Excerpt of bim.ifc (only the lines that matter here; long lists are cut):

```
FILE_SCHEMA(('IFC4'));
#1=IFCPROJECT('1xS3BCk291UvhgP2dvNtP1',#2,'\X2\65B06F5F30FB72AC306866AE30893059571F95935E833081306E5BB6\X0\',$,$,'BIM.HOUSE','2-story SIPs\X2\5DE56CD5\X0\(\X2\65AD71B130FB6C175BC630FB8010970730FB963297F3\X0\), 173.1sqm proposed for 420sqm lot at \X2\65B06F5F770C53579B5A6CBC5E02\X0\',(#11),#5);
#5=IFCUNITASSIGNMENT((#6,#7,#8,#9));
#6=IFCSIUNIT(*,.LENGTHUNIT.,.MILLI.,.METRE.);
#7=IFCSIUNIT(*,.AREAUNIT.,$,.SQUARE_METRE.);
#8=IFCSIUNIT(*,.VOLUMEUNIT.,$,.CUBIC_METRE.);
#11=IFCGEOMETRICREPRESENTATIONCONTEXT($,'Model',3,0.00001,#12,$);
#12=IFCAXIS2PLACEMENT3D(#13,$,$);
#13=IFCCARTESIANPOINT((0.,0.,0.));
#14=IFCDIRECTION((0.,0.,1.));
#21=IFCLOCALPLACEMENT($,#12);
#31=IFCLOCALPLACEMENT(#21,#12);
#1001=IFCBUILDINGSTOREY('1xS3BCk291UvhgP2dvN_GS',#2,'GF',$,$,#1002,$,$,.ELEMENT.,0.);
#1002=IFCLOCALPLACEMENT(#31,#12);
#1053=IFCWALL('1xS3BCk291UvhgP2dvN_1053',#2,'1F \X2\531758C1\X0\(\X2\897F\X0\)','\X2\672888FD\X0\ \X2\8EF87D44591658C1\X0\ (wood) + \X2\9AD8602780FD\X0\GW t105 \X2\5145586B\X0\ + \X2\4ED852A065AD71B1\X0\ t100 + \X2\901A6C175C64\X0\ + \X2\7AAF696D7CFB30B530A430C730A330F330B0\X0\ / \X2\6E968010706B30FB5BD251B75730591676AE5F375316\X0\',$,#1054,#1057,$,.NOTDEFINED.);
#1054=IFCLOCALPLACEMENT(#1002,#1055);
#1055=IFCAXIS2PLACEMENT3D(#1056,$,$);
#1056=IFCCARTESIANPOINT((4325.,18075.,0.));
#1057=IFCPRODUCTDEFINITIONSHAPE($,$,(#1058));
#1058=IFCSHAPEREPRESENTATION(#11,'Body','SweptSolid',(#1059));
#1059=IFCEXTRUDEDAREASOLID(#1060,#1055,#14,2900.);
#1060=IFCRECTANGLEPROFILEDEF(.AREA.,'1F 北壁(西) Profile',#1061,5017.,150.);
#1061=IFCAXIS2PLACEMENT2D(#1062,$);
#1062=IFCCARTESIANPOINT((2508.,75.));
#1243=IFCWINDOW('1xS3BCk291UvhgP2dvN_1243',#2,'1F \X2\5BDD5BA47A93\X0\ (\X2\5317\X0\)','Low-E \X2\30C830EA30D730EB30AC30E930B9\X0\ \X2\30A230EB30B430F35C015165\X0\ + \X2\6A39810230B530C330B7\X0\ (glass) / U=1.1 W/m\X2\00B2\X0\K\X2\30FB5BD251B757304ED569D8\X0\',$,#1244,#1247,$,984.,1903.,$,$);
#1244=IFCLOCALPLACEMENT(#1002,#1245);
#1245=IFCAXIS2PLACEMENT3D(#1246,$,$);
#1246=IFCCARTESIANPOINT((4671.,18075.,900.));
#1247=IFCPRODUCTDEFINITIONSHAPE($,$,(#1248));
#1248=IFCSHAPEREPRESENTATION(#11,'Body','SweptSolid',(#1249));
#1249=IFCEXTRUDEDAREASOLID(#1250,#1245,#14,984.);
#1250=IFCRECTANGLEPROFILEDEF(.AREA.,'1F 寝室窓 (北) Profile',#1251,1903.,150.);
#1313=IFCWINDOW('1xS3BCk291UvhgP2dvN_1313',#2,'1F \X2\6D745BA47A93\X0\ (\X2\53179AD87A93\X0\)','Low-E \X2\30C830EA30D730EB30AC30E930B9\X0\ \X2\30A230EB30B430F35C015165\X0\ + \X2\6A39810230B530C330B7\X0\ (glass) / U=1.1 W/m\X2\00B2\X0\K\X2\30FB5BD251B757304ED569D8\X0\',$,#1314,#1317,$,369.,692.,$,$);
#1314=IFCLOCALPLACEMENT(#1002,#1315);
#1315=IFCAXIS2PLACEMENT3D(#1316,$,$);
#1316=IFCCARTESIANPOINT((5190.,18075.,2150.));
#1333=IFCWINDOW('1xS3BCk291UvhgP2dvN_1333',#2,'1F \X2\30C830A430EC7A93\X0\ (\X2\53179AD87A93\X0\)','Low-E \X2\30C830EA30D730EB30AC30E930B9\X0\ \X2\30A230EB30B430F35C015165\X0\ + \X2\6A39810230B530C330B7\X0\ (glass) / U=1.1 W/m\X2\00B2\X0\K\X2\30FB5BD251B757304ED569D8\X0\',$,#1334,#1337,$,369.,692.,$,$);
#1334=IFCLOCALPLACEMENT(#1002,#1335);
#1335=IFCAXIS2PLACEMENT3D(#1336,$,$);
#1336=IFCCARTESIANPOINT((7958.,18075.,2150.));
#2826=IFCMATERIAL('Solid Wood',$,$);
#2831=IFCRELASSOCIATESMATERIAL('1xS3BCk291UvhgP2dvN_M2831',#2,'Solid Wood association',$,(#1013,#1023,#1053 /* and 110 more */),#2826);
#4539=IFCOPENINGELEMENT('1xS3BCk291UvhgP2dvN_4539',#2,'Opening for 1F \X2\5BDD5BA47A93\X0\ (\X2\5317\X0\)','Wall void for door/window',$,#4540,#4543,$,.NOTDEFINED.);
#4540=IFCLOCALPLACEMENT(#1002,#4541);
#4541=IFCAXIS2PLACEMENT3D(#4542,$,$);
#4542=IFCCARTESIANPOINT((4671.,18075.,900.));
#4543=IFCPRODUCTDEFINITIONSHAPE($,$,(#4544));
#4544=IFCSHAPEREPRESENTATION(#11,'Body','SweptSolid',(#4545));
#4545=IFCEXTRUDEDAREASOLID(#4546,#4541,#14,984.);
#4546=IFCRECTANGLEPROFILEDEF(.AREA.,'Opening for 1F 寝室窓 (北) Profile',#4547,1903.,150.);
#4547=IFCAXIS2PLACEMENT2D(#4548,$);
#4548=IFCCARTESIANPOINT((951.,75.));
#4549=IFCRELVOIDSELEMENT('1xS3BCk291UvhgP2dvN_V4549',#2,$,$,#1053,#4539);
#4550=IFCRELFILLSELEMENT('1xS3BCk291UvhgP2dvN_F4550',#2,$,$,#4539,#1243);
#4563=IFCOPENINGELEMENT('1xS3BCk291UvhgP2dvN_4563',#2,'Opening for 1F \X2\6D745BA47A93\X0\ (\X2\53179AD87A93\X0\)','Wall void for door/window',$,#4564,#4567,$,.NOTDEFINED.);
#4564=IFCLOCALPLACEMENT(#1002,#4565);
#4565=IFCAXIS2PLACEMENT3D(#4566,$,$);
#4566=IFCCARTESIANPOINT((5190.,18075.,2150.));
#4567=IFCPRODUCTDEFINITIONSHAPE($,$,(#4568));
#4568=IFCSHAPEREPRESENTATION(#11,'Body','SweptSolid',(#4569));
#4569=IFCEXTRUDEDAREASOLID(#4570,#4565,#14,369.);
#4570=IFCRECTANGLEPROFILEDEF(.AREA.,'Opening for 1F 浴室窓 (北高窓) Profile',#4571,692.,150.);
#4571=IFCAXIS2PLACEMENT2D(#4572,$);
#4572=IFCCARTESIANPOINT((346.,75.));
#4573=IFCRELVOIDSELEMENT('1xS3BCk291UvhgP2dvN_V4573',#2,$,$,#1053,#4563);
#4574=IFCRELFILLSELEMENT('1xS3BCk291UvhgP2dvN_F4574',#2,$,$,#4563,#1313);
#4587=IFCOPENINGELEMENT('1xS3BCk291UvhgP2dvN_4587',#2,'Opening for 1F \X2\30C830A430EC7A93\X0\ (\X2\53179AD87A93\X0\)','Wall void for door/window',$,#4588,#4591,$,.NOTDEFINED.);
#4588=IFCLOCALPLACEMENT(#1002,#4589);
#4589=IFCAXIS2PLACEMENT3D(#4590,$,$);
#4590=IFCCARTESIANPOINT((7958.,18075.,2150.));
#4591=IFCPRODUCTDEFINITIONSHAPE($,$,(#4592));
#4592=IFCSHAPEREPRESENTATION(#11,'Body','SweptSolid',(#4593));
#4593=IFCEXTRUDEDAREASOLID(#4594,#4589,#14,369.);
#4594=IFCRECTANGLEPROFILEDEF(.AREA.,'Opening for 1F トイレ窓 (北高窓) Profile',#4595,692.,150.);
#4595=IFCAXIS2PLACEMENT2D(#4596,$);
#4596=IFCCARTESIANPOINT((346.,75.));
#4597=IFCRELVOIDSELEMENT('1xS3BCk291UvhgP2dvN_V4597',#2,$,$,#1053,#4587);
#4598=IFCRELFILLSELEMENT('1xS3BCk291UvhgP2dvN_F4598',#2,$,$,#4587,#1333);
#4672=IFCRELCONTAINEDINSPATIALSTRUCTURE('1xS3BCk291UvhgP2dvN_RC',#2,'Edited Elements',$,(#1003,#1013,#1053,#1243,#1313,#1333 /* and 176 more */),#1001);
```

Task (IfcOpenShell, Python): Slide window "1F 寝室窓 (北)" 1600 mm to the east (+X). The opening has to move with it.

```python
import ifcopenshell
import ifcopenshell.api.geometry
import ifcopenshell.util.placement
import ifcopenshell.util.unit

model = ifcopenshell.open("bim.ifc")
unit_scale = ifcopenshell.util.unit.calculate_unit_scale(model)

window = model.by_id(1243)
opening = window.FillsVoids[0].RelatingOpeningElement
wall = opening.VoidsElements[0].RelatingBuildingElement

wall_matrix = ifcopenshell.util.placement.get_local_placement(wall.ObjectPlacement)
shift = wall_matrix[:3, 0] * 1.6 / unit_scale
before = ifcopenshell.util.placement.get_local_placement(window.ObjectPlacement)[:3, 3].copy()

# The window is not placed relative to its opening, so move both.
for product in (opening, window):
    matrix = ifcopenshell.util.placement.get_local_placement(product.ObjectPlacement)
    matrix[:3, 3] += shift
    ifcopenshell.api.geometry.edit_object_placement(model, product=product, matrix=matrix, is_si=False)

after = ifcopenshell.util.placement.get_local_placement(window.ObjectPlacement)[:3, 3]
print("window moved by", (after - before).round(3) + 0.0)

model.write("bim_v2.ifc")
```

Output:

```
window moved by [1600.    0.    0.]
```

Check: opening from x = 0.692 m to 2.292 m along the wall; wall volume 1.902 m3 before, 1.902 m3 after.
